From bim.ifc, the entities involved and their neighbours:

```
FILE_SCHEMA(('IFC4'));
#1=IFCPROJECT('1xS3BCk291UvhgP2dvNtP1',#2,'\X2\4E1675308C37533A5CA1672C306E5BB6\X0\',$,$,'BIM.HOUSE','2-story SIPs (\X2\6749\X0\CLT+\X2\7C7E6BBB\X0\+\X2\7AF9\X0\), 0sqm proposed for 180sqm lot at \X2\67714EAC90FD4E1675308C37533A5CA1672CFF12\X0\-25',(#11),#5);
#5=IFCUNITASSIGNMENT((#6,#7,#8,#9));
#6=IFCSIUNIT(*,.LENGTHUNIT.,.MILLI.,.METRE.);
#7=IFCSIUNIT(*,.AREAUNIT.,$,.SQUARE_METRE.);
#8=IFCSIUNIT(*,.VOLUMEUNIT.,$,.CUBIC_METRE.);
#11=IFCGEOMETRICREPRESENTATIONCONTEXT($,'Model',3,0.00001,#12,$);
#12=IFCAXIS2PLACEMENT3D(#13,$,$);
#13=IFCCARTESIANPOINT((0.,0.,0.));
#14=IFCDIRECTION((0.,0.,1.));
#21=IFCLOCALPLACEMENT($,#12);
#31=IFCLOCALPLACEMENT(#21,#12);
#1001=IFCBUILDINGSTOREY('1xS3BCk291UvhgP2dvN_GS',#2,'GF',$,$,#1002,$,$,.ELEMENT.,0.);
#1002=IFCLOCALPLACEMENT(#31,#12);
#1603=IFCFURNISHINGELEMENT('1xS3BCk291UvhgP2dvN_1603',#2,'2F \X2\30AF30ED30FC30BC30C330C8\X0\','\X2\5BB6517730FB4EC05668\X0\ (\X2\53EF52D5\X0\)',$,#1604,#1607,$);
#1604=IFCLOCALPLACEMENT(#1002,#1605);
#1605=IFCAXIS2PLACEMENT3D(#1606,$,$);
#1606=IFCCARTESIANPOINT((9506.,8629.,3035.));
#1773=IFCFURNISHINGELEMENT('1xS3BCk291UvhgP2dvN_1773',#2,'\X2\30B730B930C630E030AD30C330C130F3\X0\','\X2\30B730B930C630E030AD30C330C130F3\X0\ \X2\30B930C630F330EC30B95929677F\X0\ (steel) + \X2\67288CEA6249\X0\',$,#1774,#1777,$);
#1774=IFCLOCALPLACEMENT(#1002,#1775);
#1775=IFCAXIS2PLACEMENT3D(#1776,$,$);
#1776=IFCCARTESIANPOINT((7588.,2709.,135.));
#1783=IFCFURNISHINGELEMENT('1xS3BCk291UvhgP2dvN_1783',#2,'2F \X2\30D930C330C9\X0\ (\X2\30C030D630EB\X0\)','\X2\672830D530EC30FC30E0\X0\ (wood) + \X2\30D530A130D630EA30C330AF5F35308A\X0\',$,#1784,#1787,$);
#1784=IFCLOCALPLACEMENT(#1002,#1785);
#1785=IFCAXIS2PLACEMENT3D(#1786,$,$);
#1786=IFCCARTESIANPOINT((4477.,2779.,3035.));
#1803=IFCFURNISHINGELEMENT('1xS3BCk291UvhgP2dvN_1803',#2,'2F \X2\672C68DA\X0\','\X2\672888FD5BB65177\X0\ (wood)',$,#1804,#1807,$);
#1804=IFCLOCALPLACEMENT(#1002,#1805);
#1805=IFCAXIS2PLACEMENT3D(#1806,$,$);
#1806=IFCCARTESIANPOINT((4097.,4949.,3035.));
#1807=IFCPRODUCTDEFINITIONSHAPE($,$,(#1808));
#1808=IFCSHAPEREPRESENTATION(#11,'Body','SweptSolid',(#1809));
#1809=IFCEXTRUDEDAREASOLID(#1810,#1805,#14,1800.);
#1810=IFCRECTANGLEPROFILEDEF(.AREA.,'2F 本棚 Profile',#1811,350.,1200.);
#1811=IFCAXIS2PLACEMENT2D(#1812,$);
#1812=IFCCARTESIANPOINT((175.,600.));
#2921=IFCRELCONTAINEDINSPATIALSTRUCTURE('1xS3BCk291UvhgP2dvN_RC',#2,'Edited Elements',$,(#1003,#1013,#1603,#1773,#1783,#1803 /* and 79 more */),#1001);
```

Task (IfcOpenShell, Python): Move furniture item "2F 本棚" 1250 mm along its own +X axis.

```python
import ifcopenshell
import ifcopenshell.api.geometry
import ifcopenshell.util.placement
import ifcopenshell.util.unit

model = ifcopenshell.open("bim.ifc")
unit_scale = ifcopenshell.util.unit.calculate_unit_scale(model)

item = model.by_guid("1xS3BCk291UvhgP2dvN_1803")
matrix = ifcopenshell.util.placement.get_local_placement(item.ObjectPlacement)
matrix[:3, 3] += matrix[:3, 0] * 1.25 / unit_scale
ifcopenshell.api.geometry.edit_object_placement(model, product=item, matrix=matrix, is_si=False)

print(ifcopenshell.util.placement.get_local_placement(item.ObjectPlacement).round(3) + 0.0)

model.write("bim-out.ifc")
```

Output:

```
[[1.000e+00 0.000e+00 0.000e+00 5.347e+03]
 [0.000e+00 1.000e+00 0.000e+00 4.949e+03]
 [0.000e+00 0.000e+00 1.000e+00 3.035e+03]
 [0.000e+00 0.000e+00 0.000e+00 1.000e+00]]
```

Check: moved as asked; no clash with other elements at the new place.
